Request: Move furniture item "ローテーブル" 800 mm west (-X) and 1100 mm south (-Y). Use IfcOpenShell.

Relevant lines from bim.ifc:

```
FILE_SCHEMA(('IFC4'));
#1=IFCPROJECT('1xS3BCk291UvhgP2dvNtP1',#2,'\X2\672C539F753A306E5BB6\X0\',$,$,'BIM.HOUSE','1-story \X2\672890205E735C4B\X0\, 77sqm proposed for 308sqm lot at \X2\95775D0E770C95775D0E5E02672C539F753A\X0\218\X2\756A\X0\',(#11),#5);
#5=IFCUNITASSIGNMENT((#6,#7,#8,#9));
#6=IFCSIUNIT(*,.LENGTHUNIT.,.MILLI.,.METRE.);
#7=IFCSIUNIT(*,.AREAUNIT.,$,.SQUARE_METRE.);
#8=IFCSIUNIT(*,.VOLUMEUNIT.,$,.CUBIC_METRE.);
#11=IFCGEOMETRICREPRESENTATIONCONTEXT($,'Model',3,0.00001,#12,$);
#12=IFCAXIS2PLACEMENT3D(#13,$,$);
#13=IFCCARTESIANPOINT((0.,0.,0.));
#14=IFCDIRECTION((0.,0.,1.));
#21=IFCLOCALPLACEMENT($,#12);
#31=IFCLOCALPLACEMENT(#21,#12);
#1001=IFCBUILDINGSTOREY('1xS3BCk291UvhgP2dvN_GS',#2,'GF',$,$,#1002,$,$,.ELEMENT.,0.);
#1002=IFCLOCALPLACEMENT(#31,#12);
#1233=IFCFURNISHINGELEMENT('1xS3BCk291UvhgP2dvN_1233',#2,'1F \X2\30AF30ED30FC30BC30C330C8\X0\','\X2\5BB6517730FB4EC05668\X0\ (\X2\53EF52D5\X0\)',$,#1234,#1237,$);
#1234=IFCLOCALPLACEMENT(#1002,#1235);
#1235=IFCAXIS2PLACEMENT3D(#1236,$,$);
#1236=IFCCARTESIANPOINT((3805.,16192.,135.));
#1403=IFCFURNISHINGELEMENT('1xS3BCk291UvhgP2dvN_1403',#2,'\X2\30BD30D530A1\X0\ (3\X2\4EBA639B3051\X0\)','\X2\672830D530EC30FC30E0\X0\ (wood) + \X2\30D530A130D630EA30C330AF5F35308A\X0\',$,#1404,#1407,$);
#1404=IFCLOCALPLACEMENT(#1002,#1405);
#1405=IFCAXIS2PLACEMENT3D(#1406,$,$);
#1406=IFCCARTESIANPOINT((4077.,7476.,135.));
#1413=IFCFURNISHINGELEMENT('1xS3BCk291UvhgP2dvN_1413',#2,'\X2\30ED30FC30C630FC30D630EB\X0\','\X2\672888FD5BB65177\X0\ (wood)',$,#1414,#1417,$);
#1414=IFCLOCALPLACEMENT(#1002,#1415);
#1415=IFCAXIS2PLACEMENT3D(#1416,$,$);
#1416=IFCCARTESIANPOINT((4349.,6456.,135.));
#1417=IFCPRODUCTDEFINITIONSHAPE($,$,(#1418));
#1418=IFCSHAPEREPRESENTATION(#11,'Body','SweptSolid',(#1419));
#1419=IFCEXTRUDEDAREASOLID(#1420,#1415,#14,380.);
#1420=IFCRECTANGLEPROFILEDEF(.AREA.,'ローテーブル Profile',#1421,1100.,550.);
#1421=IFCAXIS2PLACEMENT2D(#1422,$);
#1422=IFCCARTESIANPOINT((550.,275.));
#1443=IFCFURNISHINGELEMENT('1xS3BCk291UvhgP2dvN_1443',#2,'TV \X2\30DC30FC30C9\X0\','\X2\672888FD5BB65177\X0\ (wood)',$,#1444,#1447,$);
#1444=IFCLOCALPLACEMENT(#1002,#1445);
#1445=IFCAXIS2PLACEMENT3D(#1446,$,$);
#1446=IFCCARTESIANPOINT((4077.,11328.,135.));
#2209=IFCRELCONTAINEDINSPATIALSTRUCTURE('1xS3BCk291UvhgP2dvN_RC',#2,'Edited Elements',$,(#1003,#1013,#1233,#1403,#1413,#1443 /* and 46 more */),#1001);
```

```python
import ifcopenshell
import ifcopenshell.api.geometry
import ifcopenshell.util.placement
import ifcopenshell.util.unit

model = ifcopenshell.open("bim.ifc")
unit_scale = ifcopenshell.util.unit.calculate_unit_scale(model)

item = model.by_id(1413)
matrix = ifcopenshell.util.placement.get_local_placement(item.ObjectPlacement)
matrix[0, 3] -= 0.8 / unit_scale
matrix[1, 3] -= 1.1 / unit_scale
ifcopenshell.api.geometry.edit_object_placement(model, product=item, matrix=matrix, is_si=False)

print(ifcopenshell.util.placement.get_local_placement(item.ObjectPlacement).round(3) + 0.0)

model.write("bim_rev.ifc")
```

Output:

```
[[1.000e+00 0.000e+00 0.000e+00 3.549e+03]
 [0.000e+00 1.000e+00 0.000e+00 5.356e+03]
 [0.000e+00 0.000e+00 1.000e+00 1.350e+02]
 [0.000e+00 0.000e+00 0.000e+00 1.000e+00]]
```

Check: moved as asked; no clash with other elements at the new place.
